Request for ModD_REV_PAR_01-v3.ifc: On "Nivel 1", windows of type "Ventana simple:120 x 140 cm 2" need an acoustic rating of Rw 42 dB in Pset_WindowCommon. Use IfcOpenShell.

First a look at what the model holds.

```python
import ifcopenshell
import ifcopenshell.util.element

model = ifcopenshell.open("ModD_REV_PAR_01-v3.ifc")
print(model.schema)
storey = next(s for s in model.by_type("IfcBuildingStorey") if s.Name == "Nivel 1")
windows = [e for e in ifcopenshell.util.element.get_decomposition(storey) if e.is_a("IfcWindow")]
seen = {}
for e in windows:
    element_type = ifcopenshell.util.element.get_type(e)
    key = (element_type.Name if element_type != e and element_type else None, ifcopenshell.util.element.get_pset(e, "Pset_WindowCommon", "AcousticRating"))
    seen[key] = seen.get(key, 0) + 1
for (name, value), count in sorted(seen.items(), key=str):
    print(count, "x", name, "|", value)
```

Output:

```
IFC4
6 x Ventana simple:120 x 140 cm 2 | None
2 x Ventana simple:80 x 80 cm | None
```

```python
import ifcopenshell
import ifcopenshell.api.pset
import ifcopenshell.util.element

model = ifcopenshell.open("ModD_REV_PAR_01-v3.ifc")

storey = next(s for s in model.by_type("IfcBuildingStorey") if s.Name == "Nivel 1")
windows = [e for e in ifcopenshell.util.element.get_decomposition(storey) if e.is_a("IfcWindow")]

count = 0
for e in windows:
    element_type = ifcopenshell.util.element.get_type(e)
    if element_type in (None, e) or element_type.Name != "Ventana simple:120 x 140 cm 2":
        continue
    # add_pset returns the element's existing set when there is one.
    pset = ifcopenshell.api.pset.add_pset(model, product=e, name="Pset_WindowCommon")
    ifcopenshell.api.pset.edit_pset(model, pset=pset, properties={"AcousticRating": "Rw 42 dB"})
    count += 1

print(count, "windows updated")

model.write("ModD_REV_PAR_01-v3_updated.ifc")
```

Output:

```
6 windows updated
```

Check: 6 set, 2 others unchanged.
